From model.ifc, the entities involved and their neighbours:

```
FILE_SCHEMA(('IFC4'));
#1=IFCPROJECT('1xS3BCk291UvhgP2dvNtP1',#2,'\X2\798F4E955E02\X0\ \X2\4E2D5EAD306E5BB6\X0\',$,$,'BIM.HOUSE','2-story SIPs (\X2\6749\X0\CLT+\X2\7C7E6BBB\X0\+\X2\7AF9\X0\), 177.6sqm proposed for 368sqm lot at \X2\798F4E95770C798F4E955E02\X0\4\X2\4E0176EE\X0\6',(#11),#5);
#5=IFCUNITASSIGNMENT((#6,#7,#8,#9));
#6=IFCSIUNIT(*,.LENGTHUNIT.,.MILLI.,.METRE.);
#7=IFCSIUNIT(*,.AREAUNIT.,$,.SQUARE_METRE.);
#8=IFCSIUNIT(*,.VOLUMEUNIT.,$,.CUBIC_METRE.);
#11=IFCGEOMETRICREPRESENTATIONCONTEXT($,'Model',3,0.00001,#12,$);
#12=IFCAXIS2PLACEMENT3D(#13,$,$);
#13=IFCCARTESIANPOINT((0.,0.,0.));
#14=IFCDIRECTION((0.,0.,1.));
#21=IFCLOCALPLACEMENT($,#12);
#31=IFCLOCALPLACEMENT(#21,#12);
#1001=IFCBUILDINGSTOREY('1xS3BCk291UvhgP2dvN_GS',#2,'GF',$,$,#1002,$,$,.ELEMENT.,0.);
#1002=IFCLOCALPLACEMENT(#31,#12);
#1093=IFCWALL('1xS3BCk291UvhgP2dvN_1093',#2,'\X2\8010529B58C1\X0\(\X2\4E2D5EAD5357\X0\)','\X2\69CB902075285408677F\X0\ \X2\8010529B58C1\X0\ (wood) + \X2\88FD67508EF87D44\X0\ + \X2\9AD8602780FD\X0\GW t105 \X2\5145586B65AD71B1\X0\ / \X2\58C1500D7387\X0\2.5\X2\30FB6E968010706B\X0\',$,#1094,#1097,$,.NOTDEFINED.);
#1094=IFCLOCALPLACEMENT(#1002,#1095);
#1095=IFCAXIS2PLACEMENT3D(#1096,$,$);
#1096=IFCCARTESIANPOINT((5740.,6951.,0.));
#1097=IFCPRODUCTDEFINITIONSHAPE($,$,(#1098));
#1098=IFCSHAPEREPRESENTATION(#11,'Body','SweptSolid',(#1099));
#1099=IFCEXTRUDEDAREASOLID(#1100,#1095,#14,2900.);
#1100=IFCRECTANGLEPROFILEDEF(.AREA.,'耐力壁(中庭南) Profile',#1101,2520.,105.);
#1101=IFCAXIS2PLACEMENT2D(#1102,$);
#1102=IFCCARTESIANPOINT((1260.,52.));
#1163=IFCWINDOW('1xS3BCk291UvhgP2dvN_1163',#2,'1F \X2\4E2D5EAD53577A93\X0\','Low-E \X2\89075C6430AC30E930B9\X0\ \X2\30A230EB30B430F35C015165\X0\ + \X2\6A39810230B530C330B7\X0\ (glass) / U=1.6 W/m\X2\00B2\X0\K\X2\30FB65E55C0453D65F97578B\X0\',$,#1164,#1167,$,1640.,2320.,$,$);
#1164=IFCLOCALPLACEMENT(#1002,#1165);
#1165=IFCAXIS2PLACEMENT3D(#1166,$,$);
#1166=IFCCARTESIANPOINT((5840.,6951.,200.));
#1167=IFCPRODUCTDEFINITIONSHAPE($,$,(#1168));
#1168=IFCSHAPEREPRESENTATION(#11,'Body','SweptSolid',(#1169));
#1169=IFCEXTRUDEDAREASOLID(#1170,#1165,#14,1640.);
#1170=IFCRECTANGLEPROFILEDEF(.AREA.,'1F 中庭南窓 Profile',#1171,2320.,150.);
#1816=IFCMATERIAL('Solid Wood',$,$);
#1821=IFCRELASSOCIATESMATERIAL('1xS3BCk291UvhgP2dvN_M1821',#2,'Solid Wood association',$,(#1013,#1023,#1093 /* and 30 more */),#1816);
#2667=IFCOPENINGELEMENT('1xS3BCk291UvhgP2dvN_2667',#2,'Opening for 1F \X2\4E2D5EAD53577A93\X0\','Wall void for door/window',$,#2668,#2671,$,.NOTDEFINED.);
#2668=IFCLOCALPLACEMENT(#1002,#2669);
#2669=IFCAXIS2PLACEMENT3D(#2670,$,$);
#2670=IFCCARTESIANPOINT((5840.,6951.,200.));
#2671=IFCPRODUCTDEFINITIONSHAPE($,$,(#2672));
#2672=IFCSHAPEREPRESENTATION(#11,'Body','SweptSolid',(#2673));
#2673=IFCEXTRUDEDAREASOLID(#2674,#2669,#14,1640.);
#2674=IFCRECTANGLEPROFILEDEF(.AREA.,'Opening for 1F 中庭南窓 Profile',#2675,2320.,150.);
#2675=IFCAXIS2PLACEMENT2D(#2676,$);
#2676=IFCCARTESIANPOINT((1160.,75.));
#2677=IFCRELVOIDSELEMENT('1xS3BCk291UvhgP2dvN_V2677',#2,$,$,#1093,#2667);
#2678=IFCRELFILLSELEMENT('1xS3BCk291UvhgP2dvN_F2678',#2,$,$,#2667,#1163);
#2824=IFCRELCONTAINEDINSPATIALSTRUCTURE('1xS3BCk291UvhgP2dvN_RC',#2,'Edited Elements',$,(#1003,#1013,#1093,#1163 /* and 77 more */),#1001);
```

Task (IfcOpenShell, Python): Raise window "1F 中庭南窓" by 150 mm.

```python
import numpy as np
import ifcopenshell
import ifcopenshell.api.geometry
import ifcopenshell.util.placement
import ifcopenshell.util.unit

model = ifcopenshell.open("model.ifc")
unit_scale = ifcopenshell.util.unit.calculate_unit_scale(model)

window = model.by_id(1163)
opening = window.FillsVoids[0].RelatingOpeningElement
dz = 0.15 / unit_scale

shift = np.array([0.0, 0.0, dz])
# The window is not placed relative to its opening, so move both.
for product in (opening, window):
    matrix = ifcopenshell.util.placement.get_local_placement(product.ObjectPlacement)
    matrix[:3, 3] += shift
    ifcopenshell.api.geometry.edit_object_placement(model, product=product, matrix=matrix, is_si=False)

print(f"moved by {dz * unit_scale:+.3f} m")

model.write("model_updated.ifc")
```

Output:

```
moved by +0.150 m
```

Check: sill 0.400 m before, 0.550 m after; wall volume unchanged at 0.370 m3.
